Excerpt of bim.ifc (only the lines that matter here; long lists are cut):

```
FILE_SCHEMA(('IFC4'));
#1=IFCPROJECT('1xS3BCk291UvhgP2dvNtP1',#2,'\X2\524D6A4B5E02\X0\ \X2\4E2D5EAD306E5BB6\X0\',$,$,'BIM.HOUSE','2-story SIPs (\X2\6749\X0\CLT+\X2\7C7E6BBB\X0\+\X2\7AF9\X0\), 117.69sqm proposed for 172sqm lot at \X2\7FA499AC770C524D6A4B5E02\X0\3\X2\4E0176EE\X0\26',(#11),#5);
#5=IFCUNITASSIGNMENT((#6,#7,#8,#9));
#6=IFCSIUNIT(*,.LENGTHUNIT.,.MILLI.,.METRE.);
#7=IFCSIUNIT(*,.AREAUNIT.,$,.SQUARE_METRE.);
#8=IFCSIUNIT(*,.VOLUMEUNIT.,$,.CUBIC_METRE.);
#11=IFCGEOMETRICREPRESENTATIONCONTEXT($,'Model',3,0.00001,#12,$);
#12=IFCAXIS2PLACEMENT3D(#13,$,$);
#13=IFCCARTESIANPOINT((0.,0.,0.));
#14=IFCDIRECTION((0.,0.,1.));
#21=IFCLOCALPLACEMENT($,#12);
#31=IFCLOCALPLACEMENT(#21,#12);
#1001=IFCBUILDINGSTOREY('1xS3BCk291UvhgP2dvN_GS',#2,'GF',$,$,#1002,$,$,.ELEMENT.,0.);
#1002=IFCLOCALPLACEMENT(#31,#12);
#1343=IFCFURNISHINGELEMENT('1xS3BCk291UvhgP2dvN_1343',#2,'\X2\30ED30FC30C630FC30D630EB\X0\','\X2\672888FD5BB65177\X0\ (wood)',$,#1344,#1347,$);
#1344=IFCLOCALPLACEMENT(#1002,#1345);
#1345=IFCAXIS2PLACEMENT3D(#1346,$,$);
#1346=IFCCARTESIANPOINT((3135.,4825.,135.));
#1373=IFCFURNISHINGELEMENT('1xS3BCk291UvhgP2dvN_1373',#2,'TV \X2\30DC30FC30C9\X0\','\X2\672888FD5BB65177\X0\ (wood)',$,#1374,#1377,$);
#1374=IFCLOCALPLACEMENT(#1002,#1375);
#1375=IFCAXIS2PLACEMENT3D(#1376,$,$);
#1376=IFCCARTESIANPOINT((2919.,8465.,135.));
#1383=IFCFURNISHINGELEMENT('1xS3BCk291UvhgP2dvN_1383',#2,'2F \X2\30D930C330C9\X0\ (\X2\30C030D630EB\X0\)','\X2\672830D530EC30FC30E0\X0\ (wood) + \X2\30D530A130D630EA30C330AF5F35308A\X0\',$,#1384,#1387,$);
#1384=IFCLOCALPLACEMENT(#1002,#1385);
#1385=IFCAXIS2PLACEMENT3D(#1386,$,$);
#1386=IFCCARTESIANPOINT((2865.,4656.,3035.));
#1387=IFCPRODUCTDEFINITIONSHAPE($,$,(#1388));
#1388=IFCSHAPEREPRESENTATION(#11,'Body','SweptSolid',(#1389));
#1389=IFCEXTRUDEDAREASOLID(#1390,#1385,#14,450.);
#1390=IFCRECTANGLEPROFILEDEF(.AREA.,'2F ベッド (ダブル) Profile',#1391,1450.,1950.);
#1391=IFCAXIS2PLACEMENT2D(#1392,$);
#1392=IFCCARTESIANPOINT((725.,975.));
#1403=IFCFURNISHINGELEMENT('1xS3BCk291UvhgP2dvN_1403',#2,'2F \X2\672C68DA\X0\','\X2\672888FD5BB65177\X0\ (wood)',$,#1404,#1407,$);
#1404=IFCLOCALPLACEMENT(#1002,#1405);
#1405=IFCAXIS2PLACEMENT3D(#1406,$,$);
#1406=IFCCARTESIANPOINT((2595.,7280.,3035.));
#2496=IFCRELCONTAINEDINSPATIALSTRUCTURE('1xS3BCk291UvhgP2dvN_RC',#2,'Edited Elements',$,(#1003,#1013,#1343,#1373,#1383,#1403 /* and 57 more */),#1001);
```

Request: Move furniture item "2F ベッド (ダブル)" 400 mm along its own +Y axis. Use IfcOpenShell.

```python
import ifcopenshell
import ifcopenshell.api.geometry
import ifcopenshell.util.placement
import ifcopenshell.util.unit

model = ifcopenshell.open("bim.ifc")
unit_scale = ifcopenshell.util.unit.calculate_unit_scale(model)

item = model.by_guid("1xS3BCk291UvhgP2dvN_1383")
matrix = ifcopenshell.util.placement.get_local_placement(item.ObjectPlacement)
matrix[:3, 3] += matrix[:3, 1] * 0.4 / unit_scale
ifcopenshell.api.geometry.edit_object_placement(model, product=item, matrix=matrix, is_si=False)

print(ifcopenshell.util.placement.get_local_placement(item.ObjectPlacement).round(3) + 0.0)

model.write("bim_updated.ifc")
```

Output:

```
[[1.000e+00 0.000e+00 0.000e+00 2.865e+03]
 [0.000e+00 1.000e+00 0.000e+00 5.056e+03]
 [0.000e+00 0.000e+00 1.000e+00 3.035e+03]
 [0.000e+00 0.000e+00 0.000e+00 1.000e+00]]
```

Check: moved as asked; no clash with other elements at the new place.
